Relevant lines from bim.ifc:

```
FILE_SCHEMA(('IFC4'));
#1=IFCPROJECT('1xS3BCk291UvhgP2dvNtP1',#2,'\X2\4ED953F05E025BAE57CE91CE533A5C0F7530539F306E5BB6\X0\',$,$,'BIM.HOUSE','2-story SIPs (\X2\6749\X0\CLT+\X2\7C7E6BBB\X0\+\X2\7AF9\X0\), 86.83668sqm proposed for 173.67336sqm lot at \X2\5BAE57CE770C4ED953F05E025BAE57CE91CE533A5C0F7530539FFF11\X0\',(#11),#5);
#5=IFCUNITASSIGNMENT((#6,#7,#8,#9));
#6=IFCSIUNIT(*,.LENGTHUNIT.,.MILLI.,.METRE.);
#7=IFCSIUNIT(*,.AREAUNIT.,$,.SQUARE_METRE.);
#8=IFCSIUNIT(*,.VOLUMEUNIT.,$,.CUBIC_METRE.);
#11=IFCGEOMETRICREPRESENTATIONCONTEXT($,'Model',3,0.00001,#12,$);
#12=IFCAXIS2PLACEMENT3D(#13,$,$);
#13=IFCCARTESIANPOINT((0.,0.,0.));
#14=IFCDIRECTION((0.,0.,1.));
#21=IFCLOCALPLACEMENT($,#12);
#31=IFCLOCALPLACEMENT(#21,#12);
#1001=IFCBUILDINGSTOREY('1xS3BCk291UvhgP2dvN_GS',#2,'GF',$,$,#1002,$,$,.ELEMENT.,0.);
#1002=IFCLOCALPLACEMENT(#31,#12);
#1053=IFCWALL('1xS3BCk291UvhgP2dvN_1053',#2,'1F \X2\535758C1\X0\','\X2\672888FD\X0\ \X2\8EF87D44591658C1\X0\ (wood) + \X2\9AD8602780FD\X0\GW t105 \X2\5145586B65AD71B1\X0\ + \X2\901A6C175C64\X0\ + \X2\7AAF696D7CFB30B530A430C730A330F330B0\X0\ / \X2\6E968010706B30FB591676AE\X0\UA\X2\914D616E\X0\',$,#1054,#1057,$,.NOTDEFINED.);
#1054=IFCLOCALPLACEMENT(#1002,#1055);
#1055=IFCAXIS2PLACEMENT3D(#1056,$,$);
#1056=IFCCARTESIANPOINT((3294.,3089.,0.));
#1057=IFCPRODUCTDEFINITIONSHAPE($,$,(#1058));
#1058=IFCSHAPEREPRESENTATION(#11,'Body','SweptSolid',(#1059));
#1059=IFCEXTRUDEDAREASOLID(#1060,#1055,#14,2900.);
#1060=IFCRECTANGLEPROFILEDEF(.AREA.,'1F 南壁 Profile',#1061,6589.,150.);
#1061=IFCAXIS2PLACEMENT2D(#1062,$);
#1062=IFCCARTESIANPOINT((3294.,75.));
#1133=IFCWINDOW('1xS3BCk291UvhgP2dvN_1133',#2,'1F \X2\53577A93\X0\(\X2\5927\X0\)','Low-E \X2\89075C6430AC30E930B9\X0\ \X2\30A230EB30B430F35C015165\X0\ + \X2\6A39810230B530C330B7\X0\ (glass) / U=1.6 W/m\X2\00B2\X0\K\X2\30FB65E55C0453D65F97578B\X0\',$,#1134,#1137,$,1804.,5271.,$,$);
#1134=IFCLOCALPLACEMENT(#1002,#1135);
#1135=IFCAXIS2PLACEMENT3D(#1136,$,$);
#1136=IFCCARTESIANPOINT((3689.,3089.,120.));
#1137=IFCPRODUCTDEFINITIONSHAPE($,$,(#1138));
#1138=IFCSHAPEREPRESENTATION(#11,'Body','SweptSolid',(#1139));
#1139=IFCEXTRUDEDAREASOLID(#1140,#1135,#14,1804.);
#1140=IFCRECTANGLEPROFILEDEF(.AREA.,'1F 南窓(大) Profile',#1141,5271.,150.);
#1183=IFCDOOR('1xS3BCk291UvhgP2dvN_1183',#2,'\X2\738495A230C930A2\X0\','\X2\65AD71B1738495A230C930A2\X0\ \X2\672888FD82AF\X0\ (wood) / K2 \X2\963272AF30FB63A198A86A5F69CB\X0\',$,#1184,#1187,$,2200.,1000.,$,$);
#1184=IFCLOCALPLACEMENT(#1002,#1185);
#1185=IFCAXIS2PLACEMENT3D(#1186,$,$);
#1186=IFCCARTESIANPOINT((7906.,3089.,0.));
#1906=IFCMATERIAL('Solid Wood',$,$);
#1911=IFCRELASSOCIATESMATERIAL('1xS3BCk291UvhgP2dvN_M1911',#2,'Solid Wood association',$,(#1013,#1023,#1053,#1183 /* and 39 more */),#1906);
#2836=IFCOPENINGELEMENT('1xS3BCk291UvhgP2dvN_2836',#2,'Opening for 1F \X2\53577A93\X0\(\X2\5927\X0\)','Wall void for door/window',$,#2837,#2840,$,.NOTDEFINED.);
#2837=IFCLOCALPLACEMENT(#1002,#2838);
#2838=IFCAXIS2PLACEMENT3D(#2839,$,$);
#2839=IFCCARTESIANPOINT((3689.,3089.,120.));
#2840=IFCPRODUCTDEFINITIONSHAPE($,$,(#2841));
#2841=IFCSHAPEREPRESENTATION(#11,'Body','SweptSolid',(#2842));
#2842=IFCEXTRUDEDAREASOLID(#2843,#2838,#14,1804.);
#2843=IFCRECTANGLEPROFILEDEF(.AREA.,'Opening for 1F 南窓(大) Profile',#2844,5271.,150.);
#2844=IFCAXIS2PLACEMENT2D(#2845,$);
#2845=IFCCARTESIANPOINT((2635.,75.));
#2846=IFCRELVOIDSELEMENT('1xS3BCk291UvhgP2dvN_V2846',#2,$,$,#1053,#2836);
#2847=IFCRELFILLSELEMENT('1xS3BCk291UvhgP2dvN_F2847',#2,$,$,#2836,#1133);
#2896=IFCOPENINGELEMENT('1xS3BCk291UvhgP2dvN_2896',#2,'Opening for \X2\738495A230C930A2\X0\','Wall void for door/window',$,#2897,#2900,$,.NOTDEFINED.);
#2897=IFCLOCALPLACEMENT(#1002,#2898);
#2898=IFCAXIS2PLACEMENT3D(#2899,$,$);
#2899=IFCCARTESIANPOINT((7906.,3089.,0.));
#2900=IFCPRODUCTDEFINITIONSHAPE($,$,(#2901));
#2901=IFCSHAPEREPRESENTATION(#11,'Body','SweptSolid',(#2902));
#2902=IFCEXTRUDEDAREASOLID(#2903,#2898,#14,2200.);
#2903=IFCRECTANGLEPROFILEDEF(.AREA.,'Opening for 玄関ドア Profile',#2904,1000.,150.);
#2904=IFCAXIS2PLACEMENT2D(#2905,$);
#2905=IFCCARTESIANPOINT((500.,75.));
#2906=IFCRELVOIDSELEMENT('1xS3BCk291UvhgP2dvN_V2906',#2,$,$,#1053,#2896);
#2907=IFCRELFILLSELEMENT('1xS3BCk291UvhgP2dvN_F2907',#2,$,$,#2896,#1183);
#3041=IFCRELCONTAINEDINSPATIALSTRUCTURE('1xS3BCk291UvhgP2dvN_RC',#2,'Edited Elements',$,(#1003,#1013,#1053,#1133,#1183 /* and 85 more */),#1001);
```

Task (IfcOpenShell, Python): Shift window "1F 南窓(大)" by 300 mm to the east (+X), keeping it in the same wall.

```python
import ifcopenshell
import ifcopenshell.api.geometry
import ifcopenshell.util.placement
import ifcopenshell.util.unit

model = ifcopenshell.open("bim.ifc")
unit_scale = ifcopenshell.util.unit.calculate_unit_scale(model)

window = model.by_guid("1xS3BCk291UvhgP2dvN_1133")
opening = window.FillsVoids[0].RelatingOpeningElement
wall = opening.VoidsElements[0].RelatingBuildingElement

wall_matrix = ifcopenshell.util.placement.get_local_placement(wall.ObjectPlacement)
shift = wall_matrix[:3, 0] * 0.3 / unit_scale
before = ifcopenshell.util.placement.get_local_placement(window.ObjectPlacement)[:3, 3].copy()

# The window is not placed relative to its opening, so move both.
for product in (opening, window):
    matrix = ifcopenshell.util.placement.get_local_placement(product.ObjectPlacement)
    matrix[:3, 3] += shift
    ifcopenshell.api.geometry.edit_object_placement(model, product=product, matrix=matrix, is_si=False)

after = ifcopenshell.util.placement.get_local_placement(window.ObjectPlacement)[:3, 3]
print("window moved by", (after - before).round(3) + 0.0)

model.write("bim-out.ifc")
```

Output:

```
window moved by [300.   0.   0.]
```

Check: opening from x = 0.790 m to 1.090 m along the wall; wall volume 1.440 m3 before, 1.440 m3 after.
